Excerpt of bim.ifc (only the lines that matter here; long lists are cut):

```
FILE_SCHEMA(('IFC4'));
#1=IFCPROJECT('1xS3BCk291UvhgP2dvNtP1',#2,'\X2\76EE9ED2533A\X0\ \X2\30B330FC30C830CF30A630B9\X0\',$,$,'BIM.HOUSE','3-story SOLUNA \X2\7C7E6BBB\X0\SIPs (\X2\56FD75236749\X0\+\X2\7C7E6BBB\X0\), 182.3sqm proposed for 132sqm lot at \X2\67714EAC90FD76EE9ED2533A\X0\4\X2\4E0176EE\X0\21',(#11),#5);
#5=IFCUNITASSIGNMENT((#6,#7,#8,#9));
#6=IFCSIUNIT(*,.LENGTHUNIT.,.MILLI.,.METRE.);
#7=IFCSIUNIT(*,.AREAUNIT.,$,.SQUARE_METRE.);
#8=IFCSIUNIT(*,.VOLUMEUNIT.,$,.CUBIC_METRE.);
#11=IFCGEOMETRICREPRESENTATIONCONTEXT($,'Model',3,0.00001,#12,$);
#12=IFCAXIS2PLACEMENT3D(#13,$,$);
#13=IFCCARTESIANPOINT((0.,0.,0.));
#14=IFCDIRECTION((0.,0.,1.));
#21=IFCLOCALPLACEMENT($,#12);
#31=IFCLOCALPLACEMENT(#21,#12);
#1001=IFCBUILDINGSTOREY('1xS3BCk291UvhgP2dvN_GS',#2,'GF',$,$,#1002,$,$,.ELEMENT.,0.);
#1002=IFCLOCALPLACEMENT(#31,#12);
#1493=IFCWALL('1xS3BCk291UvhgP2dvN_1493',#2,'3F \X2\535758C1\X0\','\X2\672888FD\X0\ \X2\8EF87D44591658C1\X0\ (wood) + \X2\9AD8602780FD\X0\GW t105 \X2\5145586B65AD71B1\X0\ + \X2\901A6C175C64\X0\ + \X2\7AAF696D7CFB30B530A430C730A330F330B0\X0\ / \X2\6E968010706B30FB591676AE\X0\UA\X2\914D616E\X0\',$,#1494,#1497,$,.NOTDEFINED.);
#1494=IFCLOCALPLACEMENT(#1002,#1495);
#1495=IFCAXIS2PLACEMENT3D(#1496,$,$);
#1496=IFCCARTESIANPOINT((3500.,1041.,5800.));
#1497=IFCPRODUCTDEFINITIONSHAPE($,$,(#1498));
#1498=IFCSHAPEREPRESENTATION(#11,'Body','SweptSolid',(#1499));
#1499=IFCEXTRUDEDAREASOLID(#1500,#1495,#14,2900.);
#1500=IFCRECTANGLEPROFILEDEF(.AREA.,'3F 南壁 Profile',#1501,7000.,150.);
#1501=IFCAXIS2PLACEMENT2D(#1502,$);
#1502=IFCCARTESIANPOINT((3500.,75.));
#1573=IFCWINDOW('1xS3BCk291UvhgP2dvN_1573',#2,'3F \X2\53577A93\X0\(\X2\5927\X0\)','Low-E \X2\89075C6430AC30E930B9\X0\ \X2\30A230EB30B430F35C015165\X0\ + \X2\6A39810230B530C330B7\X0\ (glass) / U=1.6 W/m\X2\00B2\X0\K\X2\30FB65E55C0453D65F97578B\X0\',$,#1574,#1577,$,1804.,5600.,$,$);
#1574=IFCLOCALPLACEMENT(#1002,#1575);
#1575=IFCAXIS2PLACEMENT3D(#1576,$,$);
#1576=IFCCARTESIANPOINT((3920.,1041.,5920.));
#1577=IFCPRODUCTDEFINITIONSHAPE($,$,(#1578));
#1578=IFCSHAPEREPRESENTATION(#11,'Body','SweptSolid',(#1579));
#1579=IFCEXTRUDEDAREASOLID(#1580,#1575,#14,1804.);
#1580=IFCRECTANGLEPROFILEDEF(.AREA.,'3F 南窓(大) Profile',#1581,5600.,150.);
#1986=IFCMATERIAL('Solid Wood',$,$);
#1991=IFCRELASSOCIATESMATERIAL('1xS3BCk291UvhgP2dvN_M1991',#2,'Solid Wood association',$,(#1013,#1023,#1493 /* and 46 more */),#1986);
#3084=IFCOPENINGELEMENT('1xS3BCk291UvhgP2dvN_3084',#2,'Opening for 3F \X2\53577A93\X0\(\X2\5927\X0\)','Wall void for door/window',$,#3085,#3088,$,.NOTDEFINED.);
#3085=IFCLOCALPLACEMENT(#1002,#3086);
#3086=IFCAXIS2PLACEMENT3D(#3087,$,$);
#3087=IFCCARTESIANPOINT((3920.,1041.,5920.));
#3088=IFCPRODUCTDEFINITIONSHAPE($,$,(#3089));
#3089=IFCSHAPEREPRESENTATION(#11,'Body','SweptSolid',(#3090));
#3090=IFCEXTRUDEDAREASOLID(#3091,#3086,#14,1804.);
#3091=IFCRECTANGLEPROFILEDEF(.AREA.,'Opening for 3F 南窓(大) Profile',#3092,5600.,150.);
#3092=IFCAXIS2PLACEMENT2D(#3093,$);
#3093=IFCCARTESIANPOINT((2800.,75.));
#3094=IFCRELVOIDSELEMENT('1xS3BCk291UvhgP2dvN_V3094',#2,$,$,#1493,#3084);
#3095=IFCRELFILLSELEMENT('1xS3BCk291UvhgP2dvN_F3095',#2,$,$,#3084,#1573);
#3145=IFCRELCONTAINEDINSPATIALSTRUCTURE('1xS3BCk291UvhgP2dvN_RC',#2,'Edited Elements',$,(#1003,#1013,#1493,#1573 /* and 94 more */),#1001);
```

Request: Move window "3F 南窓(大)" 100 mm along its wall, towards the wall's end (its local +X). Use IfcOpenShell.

```python
import ifcopenshell
import ifcopenshell.api.geometry
import ifcopenshell.util.placement
import ifcopenshell.util.unit

model = ifcopenshell.open("bim.ifc")
unit_scale = ifcopenshell.util.unit.calculate_unit_scale(model)

window = model.by_id(1573)
opening = window.FillsVoids[0].RelatingOpeningElement
wall = opening.VoidsElements[0].RelatingBuildingElement

wall_matrix = ifcopenshell.util.placement.get_local_placement(wall.ObjectPlacement)
shift = wall_matrix[:3, 0] * 0.1 / unit_scale
before = ifcopenshell.util.placement.get_local_placement(window.ObjectPlacement)[:3, 3].copy()

# The window is not placed relative to its opening, so move both.
for product in (opening, window):
    matrix = ifcopenshell.util.placement.get_local_placement(product.ObjectPlacement)
    matrix[:3, 3] += shift
    ifcopenshell.api.geometry.edit_object_placement(model, product=product, matrix=matrix, is_si=False)

after = ifcopenshell.util.placement.get_local_placement(window.ObjectPlacement)[:3, 3]
print("window moved by", (after - before).round(3) + 0.0)

model.write("bim_edited.ifc")
```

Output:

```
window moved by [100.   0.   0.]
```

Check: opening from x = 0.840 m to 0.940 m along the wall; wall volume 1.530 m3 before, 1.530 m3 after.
